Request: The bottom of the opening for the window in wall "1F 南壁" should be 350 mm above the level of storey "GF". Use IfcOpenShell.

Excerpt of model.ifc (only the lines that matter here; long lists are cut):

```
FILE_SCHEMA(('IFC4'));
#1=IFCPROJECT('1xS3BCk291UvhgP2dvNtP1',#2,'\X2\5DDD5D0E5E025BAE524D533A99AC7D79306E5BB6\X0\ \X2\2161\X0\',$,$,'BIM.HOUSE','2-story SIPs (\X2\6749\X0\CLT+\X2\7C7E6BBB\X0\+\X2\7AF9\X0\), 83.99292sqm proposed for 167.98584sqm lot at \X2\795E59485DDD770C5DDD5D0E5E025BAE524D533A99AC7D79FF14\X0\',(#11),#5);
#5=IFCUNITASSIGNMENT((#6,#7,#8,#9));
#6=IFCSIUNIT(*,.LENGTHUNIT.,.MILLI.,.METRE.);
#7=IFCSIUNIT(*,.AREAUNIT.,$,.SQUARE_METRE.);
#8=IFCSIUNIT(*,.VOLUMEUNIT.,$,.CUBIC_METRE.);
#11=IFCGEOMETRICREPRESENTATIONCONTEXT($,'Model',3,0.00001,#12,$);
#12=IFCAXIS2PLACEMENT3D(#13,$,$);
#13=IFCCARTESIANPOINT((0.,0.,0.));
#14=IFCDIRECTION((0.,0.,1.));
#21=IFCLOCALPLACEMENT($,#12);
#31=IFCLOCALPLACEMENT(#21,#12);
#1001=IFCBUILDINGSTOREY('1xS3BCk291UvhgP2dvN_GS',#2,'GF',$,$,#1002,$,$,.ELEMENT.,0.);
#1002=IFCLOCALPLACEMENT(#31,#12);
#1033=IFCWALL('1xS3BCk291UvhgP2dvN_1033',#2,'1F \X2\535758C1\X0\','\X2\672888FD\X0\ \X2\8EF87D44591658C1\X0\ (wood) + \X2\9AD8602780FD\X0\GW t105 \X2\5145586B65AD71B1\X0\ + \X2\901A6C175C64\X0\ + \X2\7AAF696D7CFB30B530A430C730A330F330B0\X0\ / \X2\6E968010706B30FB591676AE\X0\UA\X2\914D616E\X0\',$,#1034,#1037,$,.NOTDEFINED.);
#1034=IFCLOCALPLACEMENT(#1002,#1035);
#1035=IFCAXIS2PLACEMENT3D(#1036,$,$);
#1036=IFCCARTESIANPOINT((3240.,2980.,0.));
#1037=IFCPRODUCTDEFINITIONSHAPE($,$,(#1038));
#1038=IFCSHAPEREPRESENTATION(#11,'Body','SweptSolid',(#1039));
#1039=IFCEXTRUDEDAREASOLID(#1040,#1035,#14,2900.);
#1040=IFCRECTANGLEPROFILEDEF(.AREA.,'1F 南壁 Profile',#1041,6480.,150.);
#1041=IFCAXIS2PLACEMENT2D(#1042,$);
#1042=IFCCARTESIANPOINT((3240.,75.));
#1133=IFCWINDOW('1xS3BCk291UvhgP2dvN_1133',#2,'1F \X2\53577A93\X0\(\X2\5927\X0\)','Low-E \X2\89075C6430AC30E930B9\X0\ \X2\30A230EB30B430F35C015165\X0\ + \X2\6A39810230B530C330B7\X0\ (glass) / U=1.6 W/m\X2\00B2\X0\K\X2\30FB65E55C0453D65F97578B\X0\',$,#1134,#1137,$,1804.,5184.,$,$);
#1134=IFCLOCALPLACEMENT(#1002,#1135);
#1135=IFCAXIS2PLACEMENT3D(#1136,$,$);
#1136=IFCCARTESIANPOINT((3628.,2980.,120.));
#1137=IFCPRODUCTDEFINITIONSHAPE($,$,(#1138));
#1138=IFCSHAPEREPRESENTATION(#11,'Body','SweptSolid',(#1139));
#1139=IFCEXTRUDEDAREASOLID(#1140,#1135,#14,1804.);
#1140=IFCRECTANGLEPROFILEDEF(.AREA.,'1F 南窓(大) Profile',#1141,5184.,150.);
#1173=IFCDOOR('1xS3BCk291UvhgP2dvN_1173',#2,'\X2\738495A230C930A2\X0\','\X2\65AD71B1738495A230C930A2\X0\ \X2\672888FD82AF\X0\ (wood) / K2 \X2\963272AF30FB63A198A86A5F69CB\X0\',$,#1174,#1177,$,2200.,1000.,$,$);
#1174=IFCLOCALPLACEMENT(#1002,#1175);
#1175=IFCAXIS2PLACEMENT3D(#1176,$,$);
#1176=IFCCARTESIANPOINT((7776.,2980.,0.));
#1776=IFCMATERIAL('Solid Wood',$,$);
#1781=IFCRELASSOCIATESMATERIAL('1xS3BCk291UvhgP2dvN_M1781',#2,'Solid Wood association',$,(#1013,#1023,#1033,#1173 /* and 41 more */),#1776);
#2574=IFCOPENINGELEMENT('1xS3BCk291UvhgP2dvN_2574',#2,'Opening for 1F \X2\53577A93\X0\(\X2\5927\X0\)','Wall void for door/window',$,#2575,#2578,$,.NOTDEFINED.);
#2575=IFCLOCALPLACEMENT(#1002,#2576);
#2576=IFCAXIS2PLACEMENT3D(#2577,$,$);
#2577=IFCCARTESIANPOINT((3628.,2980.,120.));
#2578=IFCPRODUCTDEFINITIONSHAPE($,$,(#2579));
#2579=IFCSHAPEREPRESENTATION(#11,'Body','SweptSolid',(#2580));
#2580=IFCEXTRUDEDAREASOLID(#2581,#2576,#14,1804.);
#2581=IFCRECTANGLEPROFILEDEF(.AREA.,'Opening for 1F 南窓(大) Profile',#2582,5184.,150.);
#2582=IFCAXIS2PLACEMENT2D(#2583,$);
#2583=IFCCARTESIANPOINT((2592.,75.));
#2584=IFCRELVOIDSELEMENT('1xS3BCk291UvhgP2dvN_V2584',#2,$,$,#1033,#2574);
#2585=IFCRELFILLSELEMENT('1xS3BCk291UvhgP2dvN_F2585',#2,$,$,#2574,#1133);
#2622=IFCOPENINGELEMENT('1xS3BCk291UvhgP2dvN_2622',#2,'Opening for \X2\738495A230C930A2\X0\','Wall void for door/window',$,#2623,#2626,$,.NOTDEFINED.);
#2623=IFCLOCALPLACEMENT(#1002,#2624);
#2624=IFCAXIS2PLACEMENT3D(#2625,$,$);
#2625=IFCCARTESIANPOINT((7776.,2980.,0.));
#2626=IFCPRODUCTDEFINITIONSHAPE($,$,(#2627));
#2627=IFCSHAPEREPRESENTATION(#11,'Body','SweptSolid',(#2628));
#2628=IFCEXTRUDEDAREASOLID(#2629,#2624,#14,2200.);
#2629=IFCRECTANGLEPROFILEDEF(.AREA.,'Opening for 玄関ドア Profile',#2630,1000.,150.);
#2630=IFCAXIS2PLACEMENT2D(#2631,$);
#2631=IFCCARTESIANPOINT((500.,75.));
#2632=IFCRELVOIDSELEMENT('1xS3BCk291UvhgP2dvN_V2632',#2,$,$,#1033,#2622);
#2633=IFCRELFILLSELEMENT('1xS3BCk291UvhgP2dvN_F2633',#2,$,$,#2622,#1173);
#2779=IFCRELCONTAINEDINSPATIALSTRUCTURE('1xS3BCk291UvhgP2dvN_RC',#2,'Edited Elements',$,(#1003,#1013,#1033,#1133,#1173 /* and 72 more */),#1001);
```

```python
import numpy as np
import ifcopenshell
import ifcopenshell.api.geometry
import ifcopenshell.geom
import ifcopenshell.util.element
import ifcopenshell.util.placement
import ifcopenshell.util.shape
import ifcopenshell.util.unit

model = ifcopenshell.open("model.ifc")
unit_scale = ifcopenshell.util.unit.calculate_unit_scale(model)

window = model.by_guid("1xS3BCk291UvhgP2dvN_1133")
opening = window.FillsVoids[0].RelatingOpeningElement
storey = ifcopenshell.util.element.get_container(window, ifc_class="IfcBuildingStorey")
level = ifcopenshell.util.placement.get_local_placement(storey.ObjectPlacement)[2, 3]

# The opening's origin need not be at the sill, so measure its lowest point.
shape = ifcopenshell.geom.create_shape(ifcopenshell.geom.settings(), opening)
bottom = ifcopenshell.util.shape.get_shape_bottom_elevation(shape, shape.geometry) / unit_scale
dz = level + 350.0 - bottom

shift = np.array([0.0, 0.0, dz])
# The window is not placed relative to its opening, so move both.
for product in (opening, window):
    matrix = ifcopenshell.util.placement.get_local_placement(product.ObjectPlacement)
    matrix[:3, 3] += shift
    ifcopenshell.api.geometry.edit_object_placement(model, product=product, matrix=matrix, is_si=False)

print(f"moved by {dz * unit_scale:+.3f} m")

model.write("model_v2.ifc")
```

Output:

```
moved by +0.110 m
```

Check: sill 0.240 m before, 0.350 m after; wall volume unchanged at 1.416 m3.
